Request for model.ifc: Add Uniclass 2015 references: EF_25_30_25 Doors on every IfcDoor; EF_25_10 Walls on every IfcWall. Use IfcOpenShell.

First a look at what the model holds.

```python
import ifcopenshell

model = ifcopenshell.open("model.ifc")
print(model.schema)
print("classifications:", [c.Name for c in model.by_type("IfcClassification")])
for ifc_class in ("IfcDoor", "IfcRoof", "IfcStair", "IfcWall", "IfcWindow"):
    print(ifc_class, len(model.by_type(ifc_class)))
```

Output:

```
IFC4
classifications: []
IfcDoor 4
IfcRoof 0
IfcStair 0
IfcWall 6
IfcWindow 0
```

```python
import ifcopenshell
import ifcopenshell.api.classification

model = ifcopenshell.open("model.ifc")

system = ifcopenshell.api.classification.add_classification(model, classification="Uniclass 2015")

codes = {
    "IfcDoor": ("EF_25_30_25", "Doors"),
    "IfcWall": ("EF_25_10", "Walls"),
}
for ifc_class, (code, name) in codes.items():
    products = model.by_type(ifc_class)
    ifcopenshell.api.classification.add_reference(
        model, products=products, classification=system, identification=code, name=name
    )
    print(code, len(products))

model.write("model_edited.ifc")
```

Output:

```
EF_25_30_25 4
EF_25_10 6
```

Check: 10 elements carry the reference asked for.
